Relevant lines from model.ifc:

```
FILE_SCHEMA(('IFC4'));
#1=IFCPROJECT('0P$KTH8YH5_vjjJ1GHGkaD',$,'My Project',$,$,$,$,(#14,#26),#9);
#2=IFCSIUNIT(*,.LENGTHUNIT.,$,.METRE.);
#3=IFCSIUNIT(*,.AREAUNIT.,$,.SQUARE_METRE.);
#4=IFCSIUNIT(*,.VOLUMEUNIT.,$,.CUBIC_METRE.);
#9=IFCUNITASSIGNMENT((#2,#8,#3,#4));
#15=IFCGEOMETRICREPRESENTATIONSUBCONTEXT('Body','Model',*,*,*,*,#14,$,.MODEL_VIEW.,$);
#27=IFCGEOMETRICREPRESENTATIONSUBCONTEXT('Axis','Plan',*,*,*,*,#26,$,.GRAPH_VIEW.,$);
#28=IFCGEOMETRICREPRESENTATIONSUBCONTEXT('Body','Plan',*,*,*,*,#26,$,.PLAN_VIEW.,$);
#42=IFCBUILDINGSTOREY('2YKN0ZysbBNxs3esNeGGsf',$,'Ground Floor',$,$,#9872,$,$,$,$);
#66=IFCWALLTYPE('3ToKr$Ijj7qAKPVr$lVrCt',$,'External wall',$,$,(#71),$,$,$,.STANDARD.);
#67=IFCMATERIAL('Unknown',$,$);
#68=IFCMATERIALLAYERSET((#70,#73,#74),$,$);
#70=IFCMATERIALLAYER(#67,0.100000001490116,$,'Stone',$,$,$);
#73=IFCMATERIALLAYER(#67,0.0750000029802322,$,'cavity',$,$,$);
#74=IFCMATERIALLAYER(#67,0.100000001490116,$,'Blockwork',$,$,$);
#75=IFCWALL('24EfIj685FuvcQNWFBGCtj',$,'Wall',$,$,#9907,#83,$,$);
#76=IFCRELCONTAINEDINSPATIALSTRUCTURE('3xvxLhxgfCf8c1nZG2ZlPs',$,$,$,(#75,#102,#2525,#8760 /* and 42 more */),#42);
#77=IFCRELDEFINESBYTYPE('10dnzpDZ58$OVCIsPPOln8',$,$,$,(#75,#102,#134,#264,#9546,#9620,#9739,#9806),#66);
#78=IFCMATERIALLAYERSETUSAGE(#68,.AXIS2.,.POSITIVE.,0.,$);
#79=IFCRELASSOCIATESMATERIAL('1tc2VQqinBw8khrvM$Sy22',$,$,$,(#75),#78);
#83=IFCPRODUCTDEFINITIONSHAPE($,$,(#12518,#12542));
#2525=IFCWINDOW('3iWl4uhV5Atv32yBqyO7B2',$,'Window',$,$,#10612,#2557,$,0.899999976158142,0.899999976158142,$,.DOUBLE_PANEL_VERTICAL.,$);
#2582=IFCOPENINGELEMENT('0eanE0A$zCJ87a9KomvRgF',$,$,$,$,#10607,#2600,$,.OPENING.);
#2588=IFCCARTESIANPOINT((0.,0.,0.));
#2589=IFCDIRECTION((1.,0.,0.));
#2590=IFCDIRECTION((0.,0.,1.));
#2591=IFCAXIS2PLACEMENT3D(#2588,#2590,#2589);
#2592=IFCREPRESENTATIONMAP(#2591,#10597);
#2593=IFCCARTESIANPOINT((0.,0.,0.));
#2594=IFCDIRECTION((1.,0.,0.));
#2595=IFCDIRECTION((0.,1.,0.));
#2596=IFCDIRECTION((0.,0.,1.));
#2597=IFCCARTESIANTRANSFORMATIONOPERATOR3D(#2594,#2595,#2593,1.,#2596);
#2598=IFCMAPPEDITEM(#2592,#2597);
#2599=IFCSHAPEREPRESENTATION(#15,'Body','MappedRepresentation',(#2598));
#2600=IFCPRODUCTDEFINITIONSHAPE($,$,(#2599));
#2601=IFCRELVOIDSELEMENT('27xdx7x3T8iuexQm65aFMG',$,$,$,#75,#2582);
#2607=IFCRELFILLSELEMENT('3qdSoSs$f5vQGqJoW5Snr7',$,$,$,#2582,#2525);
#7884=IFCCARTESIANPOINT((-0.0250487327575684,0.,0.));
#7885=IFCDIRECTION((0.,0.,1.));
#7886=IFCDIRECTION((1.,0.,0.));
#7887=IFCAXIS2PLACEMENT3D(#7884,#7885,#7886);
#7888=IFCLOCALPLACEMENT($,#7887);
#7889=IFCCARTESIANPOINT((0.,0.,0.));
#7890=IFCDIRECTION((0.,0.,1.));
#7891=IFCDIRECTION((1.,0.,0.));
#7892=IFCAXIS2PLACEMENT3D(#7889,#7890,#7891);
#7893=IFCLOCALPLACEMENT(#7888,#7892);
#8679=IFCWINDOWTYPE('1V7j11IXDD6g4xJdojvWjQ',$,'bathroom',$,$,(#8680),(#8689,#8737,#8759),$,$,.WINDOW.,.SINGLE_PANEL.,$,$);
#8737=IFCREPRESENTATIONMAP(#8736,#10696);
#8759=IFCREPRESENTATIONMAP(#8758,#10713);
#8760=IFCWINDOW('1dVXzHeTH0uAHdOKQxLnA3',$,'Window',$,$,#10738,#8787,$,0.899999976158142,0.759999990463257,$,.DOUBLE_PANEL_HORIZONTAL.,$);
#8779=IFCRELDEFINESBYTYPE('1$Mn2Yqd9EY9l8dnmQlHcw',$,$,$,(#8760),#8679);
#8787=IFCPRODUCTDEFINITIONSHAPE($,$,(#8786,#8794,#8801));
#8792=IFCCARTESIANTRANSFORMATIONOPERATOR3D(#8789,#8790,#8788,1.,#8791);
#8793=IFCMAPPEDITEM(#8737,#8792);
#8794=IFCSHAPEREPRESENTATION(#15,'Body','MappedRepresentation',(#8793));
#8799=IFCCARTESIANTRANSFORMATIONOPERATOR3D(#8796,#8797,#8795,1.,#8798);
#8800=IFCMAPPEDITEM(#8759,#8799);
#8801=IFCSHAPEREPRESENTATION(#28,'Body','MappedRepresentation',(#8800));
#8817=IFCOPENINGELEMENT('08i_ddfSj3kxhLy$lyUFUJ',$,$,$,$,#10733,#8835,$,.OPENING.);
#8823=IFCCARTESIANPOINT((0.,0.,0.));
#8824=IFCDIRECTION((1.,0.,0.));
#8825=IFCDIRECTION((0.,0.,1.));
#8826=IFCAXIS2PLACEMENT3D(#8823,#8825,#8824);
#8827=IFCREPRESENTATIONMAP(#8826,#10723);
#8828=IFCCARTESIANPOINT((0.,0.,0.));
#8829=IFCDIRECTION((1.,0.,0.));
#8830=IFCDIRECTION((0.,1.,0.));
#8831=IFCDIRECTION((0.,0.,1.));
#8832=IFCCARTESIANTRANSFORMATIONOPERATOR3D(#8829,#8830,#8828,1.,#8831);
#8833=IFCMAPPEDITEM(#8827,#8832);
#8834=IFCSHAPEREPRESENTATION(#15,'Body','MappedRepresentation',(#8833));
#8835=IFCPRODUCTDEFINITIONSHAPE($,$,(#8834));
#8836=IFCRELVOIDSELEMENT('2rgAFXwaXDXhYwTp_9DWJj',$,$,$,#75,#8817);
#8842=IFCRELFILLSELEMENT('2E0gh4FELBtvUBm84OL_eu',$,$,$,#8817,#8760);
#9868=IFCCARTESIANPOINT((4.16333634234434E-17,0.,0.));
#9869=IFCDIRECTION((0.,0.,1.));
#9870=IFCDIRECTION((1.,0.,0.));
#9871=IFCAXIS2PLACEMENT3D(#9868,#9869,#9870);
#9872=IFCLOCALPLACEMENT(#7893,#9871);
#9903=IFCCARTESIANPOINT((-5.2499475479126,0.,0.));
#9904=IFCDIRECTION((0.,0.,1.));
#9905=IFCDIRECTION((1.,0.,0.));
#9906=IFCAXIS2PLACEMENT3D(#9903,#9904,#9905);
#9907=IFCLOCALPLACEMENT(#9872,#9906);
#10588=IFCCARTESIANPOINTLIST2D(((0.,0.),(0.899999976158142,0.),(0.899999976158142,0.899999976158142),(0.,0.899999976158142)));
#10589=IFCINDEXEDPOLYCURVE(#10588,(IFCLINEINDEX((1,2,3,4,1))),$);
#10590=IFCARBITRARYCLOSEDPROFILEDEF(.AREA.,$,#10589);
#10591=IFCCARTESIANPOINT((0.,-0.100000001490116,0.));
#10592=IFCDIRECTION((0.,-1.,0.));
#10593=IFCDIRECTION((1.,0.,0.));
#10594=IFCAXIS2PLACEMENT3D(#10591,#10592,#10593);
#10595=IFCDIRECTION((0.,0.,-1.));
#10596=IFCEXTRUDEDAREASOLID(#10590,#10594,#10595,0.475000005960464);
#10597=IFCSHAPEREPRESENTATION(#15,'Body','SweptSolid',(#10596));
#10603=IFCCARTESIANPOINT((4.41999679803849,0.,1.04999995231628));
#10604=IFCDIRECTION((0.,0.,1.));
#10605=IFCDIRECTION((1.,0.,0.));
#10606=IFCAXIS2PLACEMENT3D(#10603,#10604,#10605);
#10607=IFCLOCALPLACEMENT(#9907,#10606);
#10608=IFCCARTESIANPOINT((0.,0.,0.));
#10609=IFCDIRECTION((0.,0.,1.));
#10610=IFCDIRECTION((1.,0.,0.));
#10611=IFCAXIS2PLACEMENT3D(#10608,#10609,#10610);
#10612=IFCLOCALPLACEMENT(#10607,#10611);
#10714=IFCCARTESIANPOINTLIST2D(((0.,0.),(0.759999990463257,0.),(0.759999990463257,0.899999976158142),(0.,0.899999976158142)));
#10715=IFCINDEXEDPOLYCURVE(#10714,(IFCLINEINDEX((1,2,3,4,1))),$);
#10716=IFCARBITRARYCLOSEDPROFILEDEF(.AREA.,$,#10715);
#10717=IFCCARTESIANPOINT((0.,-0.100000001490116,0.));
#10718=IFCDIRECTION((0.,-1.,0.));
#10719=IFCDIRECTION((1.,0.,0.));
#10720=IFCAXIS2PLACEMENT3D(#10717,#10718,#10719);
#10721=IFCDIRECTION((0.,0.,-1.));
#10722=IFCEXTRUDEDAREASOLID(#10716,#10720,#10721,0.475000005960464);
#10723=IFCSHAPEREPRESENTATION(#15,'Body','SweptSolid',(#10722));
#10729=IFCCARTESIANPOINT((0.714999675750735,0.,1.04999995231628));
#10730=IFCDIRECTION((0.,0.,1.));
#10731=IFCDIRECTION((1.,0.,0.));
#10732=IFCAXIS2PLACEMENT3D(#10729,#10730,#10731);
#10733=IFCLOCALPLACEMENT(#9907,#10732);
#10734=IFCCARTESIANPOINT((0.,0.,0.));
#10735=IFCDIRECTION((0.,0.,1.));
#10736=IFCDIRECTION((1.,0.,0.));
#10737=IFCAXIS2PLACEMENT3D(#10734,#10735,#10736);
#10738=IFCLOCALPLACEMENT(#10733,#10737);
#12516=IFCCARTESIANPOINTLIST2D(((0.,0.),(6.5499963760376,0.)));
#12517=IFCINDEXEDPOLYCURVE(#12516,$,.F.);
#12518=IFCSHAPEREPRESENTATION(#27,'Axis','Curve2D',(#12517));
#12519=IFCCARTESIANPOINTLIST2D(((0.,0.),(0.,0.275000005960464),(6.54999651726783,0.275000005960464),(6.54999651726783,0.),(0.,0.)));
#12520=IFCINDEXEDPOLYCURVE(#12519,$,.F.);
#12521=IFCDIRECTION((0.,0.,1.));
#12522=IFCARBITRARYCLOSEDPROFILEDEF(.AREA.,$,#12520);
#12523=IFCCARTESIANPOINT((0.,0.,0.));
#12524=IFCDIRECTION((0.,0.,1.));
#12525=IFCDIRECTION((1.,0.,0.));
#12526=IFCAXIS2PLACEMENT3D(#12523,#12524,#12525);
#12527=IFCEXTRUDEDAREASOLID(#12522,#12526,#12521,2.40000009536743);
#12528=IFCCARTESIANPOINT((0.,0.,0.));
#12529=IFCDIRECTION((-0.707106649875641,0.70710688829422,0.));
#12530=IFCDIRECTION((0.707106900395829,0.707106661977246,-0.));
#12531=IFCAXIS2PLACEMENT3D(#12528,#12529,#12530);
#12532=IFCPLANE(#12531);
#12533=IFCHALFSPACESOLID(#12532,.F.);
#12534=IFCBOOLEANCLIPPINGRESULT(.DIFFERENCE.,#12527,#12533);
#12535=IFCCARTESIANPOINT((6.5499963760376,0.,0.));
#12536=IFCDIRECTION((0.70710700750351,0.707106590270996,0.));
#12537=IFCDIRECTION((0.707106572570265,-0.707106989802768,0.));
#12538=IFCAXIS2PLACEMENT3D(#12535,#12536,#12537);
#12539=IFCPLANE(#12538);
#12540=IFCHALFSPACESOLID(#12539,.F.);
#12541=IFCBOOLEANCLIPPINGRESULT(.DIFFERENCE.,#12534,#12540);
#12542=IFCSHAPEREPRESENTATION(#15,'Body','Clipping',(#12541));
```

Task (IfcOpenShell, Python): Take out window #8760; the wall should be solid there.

```python
import ifcopenshell
import ifcopenshell.api.feature
import ifcopenshell.api.root
import ifcopenshell.geom
import ifcopenshell.util.shape

model = ifcopenshell.open("model.ifc")
settings = ifcopenshell.geom.settings()


def volume(element):
    """Net volume in cubic metres, openings subtracted."""
    shape = ifcopenshell.geom.create_shape(settings, element)
    return ifcopenshell.util.shape.get_volume(shape.geometry)


window = model.by_guid("1dVXzHeTH0uAHdOKQxLnA3")
opening = window.FillsVoids[0].RelatingOpeningElement
wall = opening.VoidsElements[0].RelatingBuildingElement
before = volume(wall)

ifcopenshell.api.root.remove_product(model, product=window)
ifcopenshell.api.feature.remove_feature(model, feature=opening)

after = volume(wall)

print(f"wall volume {before:.3f} -> {after:.3f} m3")

model.write("model_edited.ifc")
```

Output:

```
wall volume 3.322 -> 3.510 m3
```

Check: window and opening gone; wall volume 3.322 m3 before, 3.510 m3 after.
